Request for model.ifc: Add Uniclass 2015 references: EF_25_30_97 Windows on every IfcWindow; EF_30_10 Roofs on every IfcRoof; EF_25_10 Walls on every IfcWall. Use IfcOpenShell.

First a look at what the model holds.

```python
import ifcopenshell

model = ifcopenshell.open("model.ifc")
print(model.schema)
print("classifications:", [c.Name for c in model.by_type("IfcClassification")])
for ifc_class in ("IfcDoor", "IfcRoof", "IfcStair", "IfcWall", "IfcWindow"):
    print(ifc_class, len(model.by_type(ifc_class)))
```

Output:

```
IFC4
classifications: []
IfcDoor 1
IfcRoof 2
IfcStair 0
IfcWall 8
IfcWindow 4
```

```python
import ifcopenshell
import ifcopenshell.api.classification

model = ifcopenshell.open("model.ifc")

system = ifcopenshell.api.classification.add_classification(model, classification="Uniclass 2015")

codes = {
    "IfcWindow": ("EF_25_30_97", "Windows"),
    "IfcRoof": ("EF_30_10", "Roofs"),
    "IfcWall": ("EF_25_10", "Walls"),
}
for ifc_class, (code, name) in codes.items():
    products = model.by_type(ifc_class)
    ifcopenshell.api.classification.add_reference(
        model, products=products, classification=system, identification=code, name=name
    )
    print(code, len(products))

model.write("model_edited.ifc")
```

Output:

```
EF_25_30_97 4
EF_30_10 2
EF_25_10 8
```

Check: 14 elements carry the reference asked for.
